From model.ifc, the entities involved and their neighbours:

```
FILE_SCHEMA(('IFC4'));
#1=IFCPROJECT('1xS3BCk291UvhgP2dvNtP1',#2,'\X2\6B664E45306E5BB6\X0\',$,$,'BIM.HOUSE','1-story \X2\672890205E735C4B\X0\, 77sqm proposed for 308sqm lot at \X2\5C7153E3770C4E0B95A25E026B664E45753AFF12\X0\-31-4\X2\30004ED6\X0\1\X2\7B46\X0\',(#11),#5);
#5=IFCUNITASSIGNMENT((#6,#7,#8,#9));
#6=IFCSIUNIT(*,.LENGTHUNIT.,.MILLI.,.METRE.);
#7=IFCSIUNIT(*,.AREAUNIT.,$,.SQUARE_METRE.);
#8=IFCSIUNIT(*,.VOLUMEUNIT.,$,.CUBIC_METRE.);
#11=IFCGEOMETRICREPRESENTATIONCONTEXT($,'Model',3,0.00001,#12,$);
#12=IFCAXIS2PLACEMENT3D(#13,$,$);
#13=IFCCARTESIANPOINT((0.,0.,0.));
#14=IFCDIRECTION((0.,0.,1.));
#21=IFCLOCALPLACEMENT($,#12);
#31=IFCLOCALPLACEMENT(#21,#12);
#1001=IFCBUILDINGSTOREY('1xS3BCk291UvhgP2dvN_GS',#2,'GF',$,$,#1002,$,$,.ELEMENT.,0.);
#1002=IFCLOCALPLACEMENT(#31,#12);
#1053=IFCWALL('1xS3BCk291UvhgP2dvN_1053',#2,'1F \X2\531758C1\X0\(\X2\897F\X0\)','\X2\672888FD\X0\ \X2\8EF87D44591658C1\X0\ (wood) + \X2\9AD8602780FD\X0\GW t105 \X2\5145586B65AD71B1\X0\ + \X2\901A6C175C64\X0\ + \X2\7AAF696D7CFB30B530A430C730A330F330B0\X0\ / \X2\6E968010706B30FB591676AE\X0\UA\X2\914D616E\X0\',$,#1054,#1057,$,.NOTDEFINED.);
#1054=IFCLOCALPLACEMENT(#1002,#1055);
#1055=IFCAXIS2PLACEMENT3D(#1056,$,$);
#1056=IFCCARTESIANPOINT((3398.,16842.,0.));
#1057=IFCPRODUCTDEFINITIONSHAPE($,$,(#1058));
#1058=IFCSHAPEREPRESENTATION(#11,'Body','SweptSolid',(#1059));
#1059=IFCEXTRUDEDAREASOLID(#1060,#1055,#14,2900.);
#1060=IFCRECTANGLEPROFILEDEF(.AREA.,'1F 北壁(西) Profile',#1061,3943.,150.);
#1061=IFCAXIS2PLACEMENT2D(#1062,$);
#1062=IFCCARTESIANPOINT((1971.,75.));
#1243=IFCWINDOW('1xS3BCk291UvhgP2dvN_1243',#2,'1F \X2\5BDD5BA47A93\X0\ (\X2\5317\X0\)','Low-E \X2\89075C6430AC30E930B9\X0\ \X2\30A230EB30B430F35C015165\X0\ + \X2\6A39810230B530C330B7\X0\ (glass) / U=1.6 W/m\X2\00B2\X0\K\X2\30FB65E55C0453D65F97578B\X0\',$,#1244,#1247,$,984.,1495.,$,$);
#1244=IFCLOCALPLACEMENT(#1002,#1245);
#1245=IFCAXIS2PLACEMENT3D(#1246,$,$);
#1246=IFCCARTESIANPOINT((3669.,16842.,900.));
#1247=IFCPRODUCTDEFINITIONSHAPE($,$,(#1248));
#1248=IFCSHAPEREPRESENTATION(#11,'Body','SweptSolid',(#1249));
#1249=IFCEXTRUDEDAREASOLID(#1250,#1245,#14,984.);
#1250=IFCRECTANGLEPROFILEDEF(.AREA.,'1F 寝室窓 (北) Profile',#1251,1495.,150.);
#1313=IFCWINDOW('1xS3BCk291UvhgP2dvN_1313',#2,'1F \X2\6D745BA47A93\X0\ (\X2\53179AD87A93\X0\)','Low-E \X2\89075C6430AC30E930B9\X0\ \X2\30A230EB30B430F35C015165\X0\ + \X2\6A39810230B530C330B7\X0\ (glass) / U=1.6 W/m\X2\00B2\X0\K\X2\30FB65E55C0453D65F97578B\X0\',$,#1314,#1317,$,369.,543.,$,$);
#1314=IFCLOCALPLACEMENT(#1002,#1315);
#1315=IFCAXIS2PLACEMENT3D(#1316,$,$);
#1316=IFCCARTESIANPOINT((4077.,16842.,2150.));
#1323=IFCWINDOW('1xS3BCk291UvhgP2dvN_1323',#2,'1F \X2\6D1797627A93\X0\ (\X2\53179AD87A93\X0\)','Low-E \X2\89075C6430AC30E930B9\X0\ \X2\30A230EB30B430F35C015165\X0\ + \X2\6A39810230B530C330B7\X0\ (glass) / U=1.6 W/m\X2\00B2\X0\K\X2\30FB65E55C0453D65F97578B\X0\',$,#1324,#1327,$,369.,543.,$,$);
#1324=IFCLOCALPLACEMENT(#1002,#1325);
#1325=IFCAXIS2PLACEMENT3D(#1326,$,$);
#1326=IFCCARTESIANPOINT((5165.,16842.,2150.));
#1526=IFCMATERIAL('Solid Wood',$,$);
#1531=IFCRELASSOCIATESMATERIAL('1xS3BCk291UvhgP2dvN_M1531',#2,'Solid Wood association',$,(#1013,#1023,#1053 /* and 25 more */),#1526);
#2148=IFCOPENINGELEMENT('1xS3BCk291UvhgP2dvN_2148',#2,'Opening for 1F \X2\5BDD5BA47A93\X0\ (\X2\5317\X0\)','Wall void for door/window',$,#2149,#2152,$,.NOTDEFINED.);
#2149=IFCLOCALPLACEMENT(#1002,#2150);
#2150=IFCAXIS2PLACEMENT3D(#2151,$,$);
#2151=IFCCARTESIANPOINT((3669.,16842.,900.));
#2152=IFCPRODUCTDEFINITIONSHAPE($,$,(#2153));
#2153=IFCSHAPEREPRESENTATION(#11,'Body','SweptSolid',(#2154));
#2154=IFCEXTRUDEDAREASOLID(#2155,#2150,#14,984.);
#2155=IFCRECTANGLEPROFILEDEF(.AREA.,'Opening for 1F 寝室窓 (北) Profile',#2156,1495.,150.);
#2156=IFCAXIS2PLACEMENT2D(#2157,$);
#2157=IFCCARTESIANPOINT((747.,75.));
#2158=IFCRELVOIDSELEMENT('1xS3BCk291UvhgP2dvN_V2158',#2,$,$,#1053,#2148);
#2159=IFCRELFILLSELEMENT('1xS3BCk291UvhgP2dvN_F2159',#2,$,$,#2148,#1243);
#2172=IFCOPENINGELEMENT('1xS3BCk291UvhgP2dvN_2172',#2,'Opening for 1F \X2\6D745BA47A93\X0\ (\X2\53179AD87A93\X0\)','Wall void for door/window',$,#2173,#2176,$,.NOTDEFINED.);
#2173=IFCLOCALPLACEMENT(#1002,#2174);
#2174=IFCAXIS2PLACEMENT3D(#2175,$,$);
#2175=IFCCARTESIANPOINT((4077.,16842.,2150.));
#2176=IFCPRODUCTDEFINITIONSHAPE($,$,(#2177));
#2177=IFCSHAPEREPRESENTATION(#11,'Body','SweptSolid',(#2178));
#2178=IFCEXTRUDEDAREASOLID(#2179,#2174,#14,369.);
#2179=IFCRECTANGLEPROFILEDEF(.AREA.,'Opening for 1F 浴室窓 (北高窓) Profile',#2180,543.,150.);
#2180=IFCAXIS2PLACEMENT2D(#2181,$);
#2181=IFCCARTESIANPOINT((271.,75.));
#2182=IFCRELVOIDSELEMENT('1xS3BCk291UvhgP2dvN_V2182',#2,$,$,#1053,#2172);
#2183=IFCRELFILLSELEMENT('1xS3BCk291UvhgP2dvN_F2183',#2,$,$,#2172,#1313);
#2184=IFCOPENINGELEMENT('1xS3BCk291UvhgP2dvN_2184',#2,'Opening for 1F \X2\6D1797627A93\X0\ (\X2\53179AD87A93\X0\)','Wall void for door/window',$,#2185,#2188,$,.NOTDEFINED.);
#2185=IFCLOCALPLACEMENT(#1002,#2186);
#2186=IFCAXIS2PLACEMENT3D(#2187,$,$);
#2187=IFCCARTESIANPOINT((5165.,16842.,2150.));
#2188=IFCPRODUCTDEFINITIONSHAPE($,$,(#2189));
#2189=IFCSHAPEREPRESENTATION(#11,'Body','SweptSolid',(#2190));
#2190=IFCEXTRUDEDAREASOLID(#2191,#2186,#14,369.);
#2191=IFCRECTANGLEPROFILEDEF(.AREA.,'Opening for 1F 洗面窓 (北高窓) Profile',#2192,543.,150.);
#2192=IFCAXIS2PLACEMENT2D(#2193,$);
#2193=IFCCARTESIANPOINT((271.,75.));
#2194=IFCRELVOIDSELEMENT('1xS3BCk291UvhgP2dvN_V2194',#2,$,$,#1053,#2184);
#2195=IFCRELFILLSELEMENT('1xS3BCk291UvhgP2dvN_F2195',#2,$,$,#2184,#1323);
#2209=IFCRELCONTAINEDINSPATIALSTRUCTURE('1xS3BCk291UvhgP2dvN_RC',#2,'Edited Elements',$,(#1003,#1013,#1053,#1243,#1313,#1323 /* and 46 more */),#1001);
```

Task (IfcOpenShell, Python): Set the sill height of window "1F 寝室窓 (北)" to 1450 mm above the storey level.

```python
import numpy as np
import ifcopenshell
import ifcopenshell.api.geometry
import ifcopenshell.geom
import ifcopenshell.util.element
import ifcopenshell.util.placement
import ifcopenshell.util.shape
import ifcopenshell.util.unit

model = ifcopenshell.open("model.ifc")
unit_scale = ifcopenshell.util.unit.calculate_unit_scale(model)

window = model.by_guid("1xS3BCk291UvhgP2dvN_1243")
opening = window.FillsVoids[0].RelatingOpeningElement
storey = ifcopenshell.util.element.get_container(window, ifc_class="IfcBuildingStorey")
level = ifcopenshell.util.placement.get_local_placement(storey.ObjectPlacement)[2, 3]

# The opening's origin need not be at the sill, so measure its lowest point.
shape = ifcopenshell.geom.create_shape(ifcopenshell.geom.settings(), opening)
bottom = ifcopenshell.util.shape.get_shape_bottom_elevation(shape, shape.geometry) / unit_scale
dz = level + 1.45 / unit_scale - bottom

shift = np.array([0.0, 0.0, dz])
# The window is not placed relative to its opening, so move both.
for product in (opening, window):
    matrix = ifcopenshell.util.placement.get_local_placement(product.ObjectPlacement)
    matrix[:3, 3] += shift
    ifcopenshell.api.geometry.edit_object_placement(model, product=product, matrix=matrix, is_si=False)

print(f"moved by {dz * unit_scale:+.3f} m")

model.write("model-out.ifc")
```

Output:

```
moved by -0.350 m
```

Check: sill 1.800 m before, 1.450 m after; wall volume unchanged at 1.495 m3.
